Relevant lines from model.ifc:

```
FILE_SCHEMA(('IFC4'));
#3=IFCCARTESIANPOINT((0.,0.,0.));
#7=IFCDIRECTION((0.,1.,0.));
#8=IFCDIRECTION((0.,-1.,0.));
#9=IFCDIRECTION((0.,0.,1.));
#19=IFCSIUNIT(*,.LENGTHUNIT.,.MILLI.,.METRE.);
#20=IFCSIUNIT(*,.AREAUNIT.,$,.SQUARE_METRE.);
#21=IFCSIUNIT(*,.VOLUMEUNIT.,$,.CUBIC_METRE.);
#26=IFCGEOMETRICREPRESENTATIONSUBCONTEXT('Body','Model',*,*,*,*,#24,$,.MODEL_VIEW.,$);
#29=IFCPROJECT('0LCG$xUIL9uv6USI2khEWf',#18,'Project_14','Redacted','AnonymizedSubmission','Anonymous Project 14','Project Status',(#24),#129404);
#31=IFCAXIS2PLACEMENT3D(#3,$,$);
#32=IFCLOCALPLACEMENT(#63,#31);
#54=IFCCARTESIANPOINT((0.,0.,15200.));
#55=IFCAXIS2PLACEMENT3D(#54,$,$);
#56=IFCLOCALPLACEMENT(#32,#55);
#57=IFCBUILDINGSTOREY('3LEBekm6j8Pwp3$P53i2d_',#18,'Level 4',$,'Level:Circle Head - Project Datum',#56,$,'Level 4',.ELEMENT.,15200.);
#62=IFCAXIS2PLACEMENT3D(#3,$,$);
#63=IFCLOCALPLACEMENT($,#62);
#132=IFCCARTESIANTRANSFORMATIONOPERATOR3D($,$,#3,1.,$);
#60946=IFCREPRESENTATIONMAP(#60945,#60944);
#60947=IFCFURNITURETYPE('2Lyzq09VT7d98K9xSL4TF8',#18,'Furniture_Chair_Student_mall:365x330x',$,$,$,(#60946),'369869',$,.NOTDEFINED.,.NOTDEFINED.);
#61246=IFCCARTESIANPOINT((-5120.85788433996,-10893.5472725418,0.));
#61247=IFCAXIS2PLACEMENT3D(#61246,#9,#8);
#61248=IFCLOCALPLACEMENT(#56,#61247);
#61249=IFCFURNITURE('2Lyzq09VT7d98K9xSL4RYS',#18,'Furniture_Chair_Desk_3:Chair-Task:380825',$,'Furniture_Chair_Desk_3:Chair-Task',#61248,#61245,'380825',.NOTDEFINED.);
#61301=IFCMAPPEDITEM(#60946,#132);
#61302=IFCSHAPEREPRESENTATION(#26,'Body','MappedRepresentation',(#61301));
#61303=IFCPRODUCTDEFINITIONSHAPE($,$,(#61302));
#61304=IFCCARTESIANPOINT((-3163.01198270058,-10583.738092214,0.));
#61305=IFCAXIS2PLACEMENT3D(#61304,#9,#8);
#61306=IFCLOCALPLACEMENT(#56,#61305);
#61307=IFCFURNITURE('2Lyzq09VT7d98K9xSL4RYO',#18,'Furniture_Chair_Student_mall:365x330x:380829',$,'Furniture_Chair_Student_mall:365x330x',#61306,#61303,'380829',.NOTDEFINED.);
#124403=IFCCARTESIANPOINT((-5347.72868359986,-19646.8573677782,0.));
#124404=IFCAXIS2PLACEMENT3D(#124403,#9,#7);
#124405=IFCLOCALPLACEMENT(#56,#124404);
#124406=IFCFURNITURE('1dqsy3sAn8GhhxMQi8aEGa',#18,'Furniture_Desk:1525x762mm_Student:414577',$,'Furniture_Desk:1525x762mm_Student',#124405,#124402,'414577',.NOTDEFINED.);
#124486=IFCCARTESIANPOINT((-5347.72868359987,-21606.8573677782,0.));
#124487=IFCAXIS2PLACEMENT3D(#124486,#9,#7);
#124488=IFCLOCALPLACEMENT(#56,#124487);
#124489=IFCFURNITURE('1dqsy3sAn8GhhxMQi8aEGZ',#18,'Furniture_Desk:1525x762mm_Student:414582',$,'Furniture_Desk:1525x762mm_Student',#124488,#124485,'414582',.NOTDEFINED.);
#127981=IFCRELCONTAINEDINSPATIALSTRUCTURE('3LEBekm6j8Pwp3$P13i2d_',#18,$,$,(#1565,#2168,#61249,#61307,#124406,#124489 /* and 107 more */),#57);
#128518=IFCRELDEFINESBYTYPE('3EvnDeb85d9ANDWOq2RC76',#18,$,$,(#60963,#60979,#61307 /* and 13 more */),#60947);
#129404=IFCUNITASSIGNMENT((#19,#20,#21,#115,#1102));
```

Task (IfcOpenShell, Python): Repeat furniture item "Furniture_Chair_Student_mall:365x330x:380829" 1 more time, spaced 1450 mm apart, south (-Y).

```python
import numpy as np
import ifcopenshell
import ifcopenshell.api.geometry
import ifcopenshell.api.root
import ifcopenshell.util.element
import ifcopenshell.util.placement
import ifcopenshell.util.unit

model = ifcopenshell.open("model.ifc")
unit_scale = ifcopenshell.util.unit.calculate_unit_scale(model)


def reuse_history(source, copy):
    """copy_class also copies each property set's owner history, people and application; keep the originals."""
    for rel in copy.IsDefinedBy:
        if rel.is_a("IfcRelDefinesByProperties") and (history := rel.RelatingPropertyDefinition.OwnerHistory):
            rel.RelatingPropertyDefinition.OwnerHistory = source.OwnerHistory
            ifcopenshell.util.element.remove_deep2(model, history)


source = model.by_guid("2Lyzq09VT7d98K9xSL4RYO")
base = ifcopenshell.util.placement.get_local_placement(source.ObjectPlacement)
step = np.array([0.0, -1.0, 0.0]) * 1.45 / unit_scale

for i in range(1, 2):
    copy = ifcopenshell.api.root.copy_class(model, product=source)
    copy.Representation = ifcopenshell.util.element.copy_deep(
        model, source.Representation, exclude=["IfcGeometricRepresentationContext", "IfcRepresentationMap"]
    )
    copy.Name = "Furniture_Chair_Student_mall:365x330x"
    copy.Tag = None
    reuse_history(source, copy)
    matrix = base.copy()
    matrix[:3, 3] += i * step
    print("added at", matrix[:3, 3].round(3) + 0.0)
    ifcopenshell.api.geometry.edit_object_placement(model, product=copy, matrix=matrix, is_si=False)

model.write("model_rev.ifc")
```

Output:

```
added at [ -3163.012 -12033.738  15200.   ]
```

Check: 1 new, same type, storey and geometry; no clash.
